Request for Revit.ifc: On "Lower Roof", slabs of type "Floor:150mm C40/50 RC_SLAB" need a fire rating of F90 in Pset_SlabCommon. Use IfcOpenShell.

First a look at what the model holds.

```python
import ifcopenshell
import ifcopenshell.util.element

model = ifcopenshell.open("Revit.ifc")
print(model.schema)
storey = next(s for s in model.by_type("IfcBuildingStorey") if s.Name == "Lower Roof")
slabs = [e for e in ifcopenshell.util.element.get_decomposition(storey) if e.is_a("IfcSlab")]
seen = {}
for e in slabs:
    element_type = ifcopenshell.util.element.get_type(e)
    key = (element_type.Name if element_type != e and element_type else None, ifcopenshell.util.element.get_pset(e, "Pset_SlabCommon", "FireRating"))
    seen[key] = seen.get(key, 0) + 1
for (name, value), count in sorted(seen.items(), key=str):
    print(count, "x", name, "|", value)
```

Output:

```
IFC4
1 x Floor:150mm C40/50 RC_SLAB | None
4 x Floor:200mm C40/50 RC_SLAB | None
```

```python
import ifcopenshell
import ifcopenshell.api.pset
import ifcopenshell.util.element

model = ifcopenshell.open("Revit.ifc")

storey = next(s for s in model.by_type("IfcBuildingStorey") if s.Name == "Lower Roof")
slabs = [e for e in ifcopenshell.util.element.get_decomposition(storey) if e.is_a("IfcSlab")]

count = 0
for e in slabs:
    element_type = ifcopenshell.util.element.get_type(e)
    if element_type in (None, e) or element_type.Name != "Floor:150mm C40/50 RC_SLAB":
        continue
    # add_pset returns the element's existing set when there is one.
    pset = ifcopenshell.api.pset.add_pset(model, product=e, name="Pset_SlabCommon")
    ifcopenshell.api.pset.edit_pset(model, pset=pset, properties={"FireRating": "F90"})
    count += 1

print(count, "slabs updated")

model.write("Revit_rev.ifc")
```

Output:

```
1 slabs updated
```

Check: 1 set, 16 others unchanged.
